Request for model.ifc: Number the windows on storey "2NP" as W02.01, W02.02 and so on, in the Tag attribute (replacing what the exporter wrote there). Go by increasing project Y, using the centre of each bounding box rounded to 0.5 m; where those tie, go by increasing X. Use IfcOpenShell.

First a look at what the model holds.

```python
import ifcopenshell
import ifcopenshell.util.element
import ifcopenshell.util.placement

model = ifcopenshell.open("model.ifc")
print(model.schema)
storey = next(s for s in model.by_type("IfcBuildingStorey") if s.Name == "2NP")
windows = [e for e in ifcopenshell.util.element.get_decomposition(storey) if e.is_a("IfcWindow")]
for e in sorted(windows, key=lambda e: e.id()):
    origin = ifcopenshell.util.placement.get_local_placement(e.ObjectPlacement)[:3, 3]
    print(e.id(), e.Tag, e.Name, origin.round(2) + 0.0, sep=" | ")
```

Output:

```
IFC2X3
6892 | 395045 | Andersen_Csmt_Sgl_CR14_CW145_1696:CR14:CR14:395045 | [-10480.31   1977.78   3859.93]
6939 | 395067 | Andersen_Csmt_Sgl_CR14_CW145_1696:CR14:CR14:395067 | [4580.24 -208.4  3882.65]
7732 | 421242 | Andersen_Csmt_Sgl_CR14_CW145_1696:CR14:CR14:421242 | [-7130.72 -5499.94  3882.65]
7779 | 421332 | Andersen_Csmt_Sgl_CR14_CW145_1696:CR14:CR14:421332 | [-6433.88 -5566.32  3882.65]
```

```python
import ifcopenshell
import ifcopenshell.geom
import ifcopenshell.util.element
import ifcopenshell.util.shape

model = ifcopenshell.open("model.ifc")
settings = ifcopenshell.geom.settings()
settings.set("use-world-coords", True)


def centre(element):
    shape = ifcopenshell.geom.create_shape(settings, element)
    return ifcopenshell.util.shape.get_bbox_centroid(shape.geometry)


storey = next(s for s in model.by_type("IfcBuildingStorey") if s.Name == "2NP")
windows = [e for e in ifcopenshell.util.element.get_decomposition(storey) if e.is_a("IfcWindow")]

# Insertion points can sit at a corner or the storey origin, so sort by the geometry (in metres).
centres = {e: centre(e) for e in windows}
windows.sort(key=lambda e: (round(centres[e][1] / 0.5), centres[e][0]))

for i, e in enumerate(windows, start=1):
    number = f"W02.{i:02d}"
    e.Tag = number
    print(e.id(), number)

model.write("model_v2.ifc")
```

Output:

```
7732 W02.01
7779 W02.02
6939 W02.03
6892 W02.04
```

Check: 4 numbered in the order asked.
